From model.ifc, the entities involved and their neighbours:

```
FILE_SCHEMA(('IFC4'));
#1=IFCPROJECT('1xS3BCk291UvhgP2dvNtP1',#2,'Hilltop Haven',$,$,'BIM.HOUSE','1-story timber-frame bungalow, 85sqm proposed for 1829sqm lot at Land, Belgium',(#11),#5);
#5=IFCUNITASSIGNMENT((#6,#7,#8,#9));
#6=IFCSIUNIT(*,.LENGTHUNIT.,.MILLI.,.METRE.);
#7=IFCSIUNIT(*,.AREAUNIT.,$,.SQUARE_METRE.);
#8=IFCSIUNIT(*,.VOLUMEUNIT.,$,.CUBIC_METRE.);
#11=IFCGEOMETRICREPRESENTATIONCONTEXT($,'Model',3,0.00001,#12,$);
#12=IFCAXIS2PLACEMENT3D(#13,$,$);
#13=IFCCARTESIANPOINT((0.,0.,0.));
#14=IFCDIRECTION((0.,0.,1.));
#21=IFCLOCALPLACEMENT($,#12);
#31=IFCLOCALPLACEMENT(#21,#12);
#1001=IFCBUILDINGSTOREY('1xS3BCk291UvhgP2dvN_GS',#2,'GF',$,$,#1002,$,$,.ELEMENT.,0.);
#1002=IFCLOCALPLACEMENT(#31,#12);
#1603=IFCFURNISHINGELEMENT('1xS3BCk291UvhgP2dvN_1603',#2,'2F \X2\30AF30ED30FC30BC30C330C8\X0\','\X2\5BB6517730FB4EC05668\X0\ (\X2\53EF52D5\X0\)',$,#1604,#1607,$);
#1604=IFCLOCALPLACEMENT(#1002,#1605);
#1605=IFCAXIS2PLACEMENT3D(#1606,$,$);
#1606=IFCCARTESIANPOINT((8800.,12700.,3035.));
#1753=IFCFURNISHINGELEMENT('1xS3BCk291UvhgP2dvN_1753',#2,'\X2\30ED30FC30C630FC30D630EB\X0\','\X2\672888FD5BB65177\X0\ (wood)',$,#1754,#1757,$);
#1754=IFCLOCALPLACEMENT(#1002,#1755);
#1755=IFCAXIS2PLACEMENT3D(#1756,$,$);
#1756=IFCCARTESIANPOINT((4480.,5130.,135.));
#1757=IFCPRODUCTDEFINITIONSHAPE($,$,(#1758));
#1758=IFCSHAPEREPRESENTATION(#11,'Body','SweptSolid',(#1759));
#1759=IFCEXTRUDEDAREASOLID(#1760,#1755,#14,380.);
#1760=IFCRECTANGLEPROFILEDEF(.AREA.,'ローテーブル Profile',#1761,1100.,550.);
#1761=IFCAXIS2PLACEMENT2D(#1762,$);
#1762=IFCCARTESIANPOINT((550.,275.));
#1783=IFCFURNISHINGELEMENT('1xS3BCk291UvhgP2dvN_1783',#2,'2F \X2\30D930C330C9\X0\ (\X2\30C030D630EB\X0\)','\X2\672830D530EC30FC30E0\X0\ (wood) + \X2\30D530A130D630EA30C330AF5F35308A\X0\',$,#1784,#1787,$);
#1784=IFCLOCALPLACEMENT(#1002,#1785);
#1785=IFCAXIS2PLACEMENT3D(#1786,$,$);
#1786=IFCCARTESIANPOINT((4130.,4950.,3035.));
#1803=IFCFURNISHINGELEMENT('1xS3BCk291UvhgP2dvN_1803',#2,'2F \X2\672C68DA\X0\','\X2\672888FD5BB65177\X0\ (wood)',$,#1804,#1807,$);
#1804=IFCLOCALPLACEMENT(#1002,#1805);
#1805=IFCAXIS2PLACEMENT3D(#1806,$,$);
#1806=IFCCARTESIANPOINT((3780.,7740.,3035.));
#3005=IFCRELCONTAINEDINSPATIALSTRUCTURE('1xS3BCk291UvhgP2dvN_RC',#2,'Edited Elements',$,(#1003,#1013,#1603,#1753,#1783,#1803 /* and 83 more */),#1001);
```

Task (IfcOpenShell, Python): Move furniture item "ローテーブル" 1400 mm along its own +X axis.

```python
import ifcopenshell
import ifcopenshell.api.geometry
import ifcopenshell.util.placement
import ifcopenshell.util.unit

model = ifcopenshell.open("model.ifc")
unit_scale = ifcopenshell.util.unit.calculate_unit_scale(model)

item = model.by_guid("1xS3BCk291UvhgP2dvN_1753")
matrix = ifcopenshell.util.placement.get_local_placement(item.ObjectPlacement)
matrix[:3, 3] += matrix[:3, 0] * 1.4 / unit_scale
ifcopenshell.api.geometry.edit_object_placement(model, product=item, matrix=matrix, is_si=False)

print(ifcopenshell.util.placement.get_local_placement(item.ObjectPlacement).round(3) + 0.0)

model.write("model_edited.ifc")
```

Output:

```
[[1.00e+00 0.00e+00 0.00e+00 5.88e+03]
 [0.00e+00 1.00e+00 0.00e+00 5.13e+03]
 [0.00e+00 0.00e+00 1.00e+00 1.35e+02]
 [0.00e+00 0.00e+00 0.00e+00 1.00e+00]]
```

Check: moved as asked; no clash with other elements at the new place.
